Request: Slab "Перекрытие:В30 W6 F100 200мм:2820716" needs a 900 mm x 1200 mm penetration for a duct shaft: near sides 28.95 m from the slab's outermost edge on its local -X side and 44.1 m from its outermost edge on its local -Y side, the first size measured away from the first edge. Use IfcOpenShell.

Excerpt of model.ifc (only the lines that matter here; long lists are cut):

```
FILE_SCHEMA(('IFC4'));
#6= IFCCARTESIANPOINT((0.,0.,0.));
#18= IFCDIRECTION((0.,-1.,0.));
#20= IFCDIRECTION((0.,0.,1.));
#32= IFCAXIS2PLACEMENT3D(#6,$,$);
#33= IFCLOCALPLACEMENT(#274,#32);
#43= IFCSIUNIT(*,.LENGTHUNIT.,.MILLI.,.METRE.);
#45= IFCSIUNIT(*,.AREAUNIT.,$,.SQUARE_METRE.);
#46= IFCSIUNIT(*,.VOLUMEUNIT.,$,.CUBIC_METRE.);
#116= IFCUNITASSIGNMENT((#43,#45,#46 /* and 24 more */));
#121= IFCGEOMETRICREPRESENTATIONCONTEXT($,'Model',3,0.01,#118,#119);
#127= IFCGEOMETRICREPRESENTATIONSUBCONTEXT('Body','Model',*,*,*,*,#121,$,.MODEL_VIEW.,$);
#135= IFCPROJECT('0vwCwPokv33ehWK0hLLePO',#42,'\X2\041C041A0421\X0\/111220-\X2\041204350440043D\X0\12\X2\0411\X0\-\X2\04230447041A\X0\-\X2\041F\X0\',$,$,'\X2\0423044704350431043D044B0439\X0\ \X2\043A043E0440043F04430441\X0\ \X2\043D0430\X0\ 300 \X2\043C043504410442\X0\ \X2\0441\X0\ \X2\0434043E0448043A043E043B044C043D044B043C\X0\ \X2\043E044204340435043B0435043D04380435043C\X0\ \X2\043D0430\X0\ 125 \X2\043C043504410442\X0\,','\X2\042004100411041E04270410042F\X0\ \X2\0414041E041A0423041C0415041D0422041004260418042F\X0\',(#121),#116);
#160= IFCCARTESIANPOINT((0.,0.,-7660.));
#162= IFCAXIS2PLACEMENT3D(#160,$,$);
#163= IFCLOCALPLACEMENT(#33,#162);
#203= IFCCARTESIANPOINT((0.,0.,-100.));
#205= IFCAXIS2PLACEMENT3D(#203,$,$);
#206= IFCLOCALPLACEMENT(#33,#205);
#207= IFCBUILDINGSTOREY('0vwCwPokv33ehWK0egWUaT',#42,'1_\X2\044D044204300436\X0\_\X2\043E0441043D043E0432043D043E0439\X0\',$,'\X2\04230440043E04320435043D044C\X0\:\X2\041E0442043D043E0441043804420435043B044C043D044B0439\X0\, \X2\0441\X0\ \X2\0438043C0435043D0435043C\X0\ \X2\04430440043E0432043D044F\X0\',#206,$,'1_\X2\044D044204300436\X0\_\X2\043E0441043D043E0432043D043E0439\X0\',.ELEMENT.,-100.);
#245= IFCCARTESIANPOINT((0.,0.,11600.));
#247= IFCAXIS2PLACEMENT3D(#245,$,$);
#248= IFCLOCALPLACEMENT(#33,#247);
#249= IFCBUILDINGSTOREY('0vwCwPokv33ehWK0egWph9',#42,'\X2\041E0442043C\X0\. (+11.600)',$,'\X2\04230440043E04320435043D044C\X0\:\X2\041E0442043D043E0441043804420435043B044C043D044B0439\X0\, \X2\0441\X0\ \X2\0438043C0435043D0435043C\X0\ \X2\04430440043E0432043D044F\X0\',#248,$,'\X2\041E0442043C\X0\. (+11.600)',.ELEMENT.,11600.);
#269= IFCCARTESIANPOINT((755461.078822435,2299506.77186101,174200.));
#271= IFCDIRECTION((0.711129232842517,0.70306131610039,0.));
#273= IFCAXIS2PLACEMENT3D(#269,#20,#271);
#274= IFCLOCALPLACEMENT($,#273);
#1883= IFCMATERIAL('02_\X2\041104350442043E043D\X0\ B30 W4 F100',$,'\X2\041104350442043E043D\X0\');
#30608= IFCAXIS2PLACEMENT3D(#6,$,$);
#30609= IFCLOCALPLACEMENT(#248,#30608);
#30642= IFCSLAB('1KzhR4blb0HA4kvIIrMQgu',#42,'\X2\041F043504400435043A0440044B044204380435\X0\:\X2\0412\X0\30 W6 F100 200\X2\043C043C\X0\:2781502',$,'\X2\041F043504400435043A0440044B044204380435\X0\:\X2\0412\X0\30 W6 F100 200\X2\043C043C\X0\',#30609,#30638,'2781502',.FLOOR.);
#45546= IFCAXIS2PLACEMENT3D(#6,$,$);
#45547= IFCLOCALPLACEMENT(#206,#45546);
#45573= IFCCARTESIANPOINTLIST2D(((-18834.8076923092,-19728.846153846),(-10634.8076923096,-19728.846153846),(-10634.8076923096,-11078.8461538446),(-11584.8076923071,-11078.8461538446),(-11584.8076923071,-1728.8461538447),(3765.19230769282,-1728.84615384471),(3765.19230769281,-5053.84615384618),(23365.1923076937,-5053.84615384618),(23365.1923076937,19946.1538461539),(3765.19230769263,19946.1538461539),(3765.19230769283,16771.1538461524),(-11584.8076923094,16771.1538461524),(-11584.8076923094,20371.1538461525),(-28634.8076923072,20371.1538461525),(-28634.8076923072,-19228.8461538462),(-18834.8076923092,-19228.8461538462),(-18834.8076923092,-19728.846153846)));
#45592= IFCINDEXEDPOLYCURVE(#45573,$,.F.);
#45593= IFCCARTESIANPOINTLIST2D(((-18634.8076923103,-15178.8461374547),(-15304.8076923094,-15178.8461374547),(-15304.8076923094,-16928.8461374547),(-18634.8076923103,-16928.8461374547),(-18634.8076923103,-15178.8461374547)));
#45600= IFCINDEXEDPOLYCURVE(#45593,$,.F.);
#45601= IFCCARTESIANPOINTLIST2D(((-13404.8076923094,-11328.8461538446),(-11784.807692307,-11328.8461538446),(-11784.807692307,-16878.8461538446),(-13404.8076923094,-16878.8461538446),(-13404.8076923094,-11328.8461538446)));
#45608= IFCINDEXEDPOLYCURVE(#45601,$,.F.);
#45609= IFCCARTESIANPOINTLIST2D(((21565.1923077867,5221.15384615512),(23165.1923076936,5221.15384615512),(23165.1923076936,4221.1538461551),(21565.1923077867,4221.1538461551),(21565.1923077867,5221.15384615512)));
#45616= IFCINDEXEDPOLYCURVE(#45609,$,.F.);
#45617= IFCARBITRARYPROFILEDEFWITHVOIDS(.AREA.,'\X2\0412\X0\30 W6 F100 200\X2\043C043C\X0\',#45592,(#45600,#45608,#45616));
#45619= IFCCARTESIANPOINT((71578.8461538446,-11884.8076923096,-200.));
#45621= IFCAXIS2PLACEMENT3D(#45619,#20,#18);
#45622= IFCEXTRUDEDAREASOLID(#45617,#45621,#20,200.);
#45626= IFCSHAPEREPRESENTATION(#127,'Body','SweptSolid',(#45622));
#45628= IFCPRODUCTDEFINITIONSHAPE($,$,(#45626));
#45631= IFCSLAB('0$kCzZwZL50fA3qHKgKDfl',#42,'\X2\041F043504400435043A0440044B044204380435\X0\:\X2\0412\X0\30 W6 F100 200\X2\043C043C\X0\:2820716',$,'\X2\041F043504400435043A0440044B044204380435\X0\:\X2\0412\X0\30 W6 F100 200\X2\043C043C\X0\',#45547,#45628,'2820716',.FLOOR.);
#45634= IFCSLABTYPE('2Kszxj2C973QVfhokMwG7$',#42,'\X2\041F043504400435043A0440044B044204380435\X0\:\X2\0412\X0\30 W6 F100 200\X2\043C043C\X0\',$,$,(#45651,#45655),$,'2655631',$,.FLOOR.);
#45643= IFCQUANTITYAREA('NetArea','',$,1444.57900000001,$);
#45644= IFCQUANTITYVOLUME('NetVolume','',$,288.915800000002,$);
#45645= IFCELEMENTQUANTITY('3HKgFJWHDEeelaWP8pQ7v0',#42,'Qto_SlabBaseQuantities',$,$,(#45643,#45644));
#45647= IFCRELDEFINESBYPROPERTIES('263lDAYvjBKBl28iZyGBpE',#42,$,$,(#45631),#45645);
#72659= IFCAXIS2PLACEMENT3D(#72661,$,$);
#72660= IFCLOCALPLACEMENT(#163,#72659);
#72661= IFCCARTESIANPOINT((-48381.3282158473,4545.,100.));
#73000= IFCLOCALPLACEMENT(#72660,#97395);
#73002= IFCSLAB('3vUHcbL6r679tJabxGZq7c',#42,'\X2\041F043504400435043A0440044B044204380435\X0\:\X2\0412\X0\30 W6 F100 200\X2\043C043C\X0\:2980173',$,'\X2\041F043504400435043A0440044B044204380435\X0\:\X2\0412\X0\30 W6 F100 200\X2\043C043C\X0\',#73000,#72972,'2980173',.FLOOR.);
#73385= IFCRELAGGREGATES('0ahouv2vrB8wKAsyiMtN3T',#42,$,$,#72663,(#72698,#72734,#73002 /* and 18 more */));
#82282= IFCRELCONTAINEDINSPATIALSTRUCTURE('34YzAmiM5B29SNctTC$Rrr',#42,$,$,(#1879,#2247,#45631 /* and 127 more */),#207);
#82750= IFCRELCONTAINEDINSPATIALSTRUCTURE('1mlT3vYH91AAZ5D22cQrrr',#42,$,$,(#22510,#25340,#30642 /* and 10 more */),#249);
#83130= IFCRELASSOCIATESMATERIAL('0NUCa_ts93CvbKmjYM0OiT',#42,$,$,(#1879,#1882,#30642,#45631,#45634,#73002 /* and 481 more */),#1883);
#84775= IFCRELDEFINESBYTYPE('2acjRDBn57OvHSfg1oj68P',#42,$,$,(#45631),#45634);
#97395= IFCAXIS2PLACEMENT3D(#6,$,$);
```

```python
import numpy as np
import ifcopenshell
import ifcopenshell.api.feature
import ifcopenshell.api.geometry
import ifcopenshell.api.pset
import ifcopenshell.api.root
import ifcopenshell.geom
import ifcopenshell.util.element
import ifcopenshell.util.placement
import ifcopenshell.util.representation
import ifcopenshell.util.shape
import ifcopenshell.util.unit

model = ifcopenshell.open("model.ifc")
unit_scale = ifcopenshell.util.unit.calculate_unit_scale(model)
area_scale = ifcopenshell.util.unit.calculate_unit_scale(model, "AREAUNIT")
volume_scale = ifcopenshell.util.unit.calculate_unit_scale(model, "VOLUMEUNIT")
settings = ifcopenshell.geom.settings()


def volume(element):
    """Net volume in cubic metres, openings subtracted."""
    shape = ifcopenshell.geom.create_shape(settings, element)
    return ifcopenshell.util.shape.get_volume(shape.geometry)


slab = model.by_guid("0$kCzZwZL50fA3qHKgKDfl")
before = volume(slab)

# Extent in the slab's own axes, in metres. The edges named are its -X and -Y sides.
slab_shape = ifcopenshell.geom.create_shape(settings, slab)
vertices = ifcopenshell.util.shape.get_vertices(slab_shape.geometry)
x_min, y_min, bottom = vertices.min(axis=0)
top = vertices[:, 2].max()

opening = ifcopenshell.api.root.create_entity(model, ifc_class="IfcOpeningElement", name="Duct shaft opening", predefined_type="OPENING")
context = ifcopenshell.util.representation.get_context(model, "Model", "Body", "MODEL_VIEW")
width, depth = 0.9, 1.2
outline = [(0.0, 0.0), (width, 0.0), (width, depth), (0.0, depth), (0.0, 0.0)]
# Overshoot both faces by 50 mm so the cut is clean.
shape = ifcopenshell.api.geometry.add_slab_representation(
    model, context=context, depth=top - bottom + 0.1, polyline=outline
)
ifcopenshell.api.geometry.assign_representation(model, product=opening, representation=shape)

matrix = ifcopenshell.util.placement.get_local_placement(slab.ObjectPlacement)
matrix[:, 3] = matrix @ np.append(np.array([x_min + 28.95, y_min + 44.1, bottom - 0.05]) / unit_scale, 1.0)
ifcopenshell.api.geometry.edit_object_placement(model, product=opening, matrix=matrix, is_si=False)
ifcopenshell.api.feature.add_feature(model, feature=opening, element=slab)

after = volume(slab)

# Update the slab's stored quantities.
qto = model.by_id(ifcopenshell.util.element.get_pset(slab, "Qto_SlabBaseQuantities", should_inherit=False)["id"])
ifcopenshell.api.pset.edit_qto(model, qto=qto, properties={
    "NetArea": after / (top - bottom) / area_scale,
    "NetVolume": after / volume_scale,
})

print(f"slab volume {before:.3f} -> {after:.3f} m3")

model.write("model_updated.ifc")
```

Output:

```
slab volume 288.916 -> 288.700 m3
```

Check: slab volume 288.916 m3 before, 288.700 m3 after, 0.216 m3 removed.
